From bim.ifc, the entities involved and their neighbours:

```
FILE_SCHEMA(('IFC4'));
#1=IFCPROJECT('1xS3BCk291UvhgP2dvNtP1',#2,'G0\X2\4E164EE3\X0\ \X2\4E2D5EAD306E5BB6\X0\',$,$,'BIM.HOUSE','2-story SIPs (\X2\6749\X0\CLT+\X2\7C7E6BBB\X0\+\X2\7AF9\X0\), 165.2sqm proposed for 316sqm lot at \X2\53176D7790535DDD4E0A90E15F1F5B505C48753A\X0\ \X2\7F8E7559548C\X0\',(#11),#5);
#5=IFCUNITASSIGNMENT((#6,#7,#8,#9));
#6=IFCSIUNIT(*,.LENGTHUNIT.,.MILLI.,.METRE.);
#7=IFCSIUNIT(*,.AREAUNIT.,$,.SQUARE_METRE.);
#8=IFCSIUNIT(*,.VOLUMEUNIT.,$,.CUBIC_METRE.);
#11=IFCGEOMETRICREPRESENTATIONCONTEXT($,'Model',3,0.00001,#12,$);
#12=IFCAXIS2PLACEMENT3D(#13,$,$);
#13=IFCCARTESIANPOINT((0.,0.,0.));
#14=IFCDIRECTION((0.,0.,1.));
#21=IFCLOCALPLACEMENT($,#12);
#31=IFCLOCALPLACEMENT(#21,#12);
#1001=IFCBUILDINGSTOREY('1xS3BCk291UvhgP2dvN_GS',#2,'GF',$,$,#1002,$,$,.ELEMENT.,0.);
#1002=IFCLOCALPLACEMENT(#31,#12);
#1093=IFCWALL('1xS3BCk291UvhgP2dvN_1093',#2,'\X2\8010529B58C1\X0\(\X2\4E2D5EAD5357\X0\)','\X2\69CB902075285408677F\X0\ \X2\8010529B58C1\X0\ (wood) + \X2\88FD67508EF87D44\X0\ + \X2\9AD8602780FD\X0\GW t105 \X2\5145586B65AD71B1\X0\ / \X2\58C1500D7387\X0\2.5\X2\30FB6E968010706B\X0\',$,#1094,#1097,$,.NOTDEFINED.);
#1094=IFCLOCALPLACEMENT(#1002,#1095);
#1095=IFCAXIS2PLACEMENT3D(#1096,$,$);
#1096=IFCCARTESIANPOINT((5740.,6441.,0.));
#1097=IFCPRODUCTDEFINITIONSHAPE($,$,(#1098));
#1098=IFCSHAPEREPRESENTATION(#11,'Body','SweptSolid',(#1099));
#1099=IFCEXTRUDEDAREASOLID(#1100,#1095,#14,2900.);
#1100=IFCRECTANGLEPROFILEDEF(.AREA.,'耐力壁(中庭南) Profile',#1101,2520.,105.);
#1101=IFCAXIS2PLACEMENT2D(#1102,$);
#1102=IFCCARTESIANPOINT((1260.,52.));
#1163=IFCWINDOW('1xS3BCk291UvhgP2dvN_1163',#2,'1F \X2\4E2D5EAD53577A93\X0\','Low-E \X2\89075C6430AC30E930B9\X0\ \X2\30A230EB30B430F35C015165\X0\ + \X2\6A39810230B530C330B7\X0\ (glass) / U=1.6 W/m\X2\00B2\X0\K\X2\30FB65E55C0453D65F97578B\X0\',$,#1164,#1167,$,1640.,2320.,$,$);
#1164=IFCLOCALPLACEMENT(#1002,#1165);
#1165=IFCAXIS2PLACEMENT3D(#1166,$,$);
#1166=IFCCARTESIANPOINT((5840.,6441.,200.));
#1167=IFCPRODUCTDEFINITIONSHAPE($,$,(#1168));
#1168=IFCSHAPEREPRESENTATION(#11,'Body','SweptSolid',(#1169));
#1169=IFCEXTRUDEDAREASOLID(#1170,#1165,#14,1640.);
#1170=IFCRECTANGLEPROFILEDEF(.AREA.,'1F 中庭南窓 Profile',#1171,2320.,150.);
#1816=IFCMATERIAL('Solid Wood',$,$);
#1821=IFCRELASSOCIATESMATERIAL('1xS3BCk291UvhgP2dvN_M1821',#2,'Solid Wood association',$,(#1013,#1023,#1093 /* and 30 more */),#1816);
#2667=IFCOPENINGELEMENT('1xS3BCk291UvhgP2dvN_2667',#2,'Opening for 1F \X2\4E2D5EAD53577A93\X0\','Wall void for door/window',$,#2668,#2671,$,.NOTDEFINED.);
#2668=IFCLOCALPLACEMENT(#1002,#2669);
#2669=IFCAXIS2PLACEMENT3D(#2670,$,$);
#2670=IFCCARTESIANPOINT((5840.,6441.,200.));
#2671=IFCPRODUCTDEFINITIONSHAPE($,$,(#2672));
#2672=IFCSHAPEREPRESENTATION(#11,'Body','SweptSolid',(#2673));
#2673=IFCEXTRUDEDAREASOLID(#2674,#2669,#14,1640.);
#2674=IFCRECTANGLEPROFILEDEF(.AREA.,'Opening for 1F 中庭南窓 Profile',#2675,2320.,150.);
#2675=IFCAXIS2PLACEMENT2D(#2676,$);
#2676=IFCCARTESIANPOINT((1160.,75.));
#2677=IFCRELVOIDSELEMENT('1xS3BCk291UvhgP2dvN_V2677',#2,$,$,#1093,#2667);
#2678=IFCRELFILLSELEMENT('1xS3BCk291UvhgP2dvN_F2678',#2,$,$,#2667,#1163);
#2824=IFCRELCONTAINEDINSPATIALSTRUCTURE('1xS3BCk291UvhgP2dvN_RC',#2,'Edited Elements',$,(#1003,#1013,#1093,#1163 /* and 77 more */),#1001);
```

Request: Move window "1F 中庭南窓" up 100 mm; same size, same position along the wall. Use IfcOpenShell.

```python
import numpy as np
import ifcopenshell
import ifcopenshell.api.geometry
import ifcopenshell.util.placement
import ifcopenshell.util.unit

model = ifcopenshell.open("bim.ifc")
unit_scale = ifcopenshell.util.unit.calculate_unit_scale(model)

window = model.by_guid("1xS3BCk291UvhgP2dvN_1163")
opening = window.FillsVoids[0].RelatingOpeningElement
dz = 0.1 / unit_scale

shift = np.array([0.0, 0.0, dz])
# The window is not placed relative to its opening, so move both.
for product in (opening, window):
    matrix = ifcopenshell.util.placement.get_local_placement(product.ObjectPlacement)
    matrix[:3, 3] += shift
    ifcopenshell.api.geometry.edit_object_placement(model, product=product, matrix=matrix, is_si=False)

print(f"moved by {dz * unit_scale:+.3f} m")

model.write("bim_rev.ifc")
```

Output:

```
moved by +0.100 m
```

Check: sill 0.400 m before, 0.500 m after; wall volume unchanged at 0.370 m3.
